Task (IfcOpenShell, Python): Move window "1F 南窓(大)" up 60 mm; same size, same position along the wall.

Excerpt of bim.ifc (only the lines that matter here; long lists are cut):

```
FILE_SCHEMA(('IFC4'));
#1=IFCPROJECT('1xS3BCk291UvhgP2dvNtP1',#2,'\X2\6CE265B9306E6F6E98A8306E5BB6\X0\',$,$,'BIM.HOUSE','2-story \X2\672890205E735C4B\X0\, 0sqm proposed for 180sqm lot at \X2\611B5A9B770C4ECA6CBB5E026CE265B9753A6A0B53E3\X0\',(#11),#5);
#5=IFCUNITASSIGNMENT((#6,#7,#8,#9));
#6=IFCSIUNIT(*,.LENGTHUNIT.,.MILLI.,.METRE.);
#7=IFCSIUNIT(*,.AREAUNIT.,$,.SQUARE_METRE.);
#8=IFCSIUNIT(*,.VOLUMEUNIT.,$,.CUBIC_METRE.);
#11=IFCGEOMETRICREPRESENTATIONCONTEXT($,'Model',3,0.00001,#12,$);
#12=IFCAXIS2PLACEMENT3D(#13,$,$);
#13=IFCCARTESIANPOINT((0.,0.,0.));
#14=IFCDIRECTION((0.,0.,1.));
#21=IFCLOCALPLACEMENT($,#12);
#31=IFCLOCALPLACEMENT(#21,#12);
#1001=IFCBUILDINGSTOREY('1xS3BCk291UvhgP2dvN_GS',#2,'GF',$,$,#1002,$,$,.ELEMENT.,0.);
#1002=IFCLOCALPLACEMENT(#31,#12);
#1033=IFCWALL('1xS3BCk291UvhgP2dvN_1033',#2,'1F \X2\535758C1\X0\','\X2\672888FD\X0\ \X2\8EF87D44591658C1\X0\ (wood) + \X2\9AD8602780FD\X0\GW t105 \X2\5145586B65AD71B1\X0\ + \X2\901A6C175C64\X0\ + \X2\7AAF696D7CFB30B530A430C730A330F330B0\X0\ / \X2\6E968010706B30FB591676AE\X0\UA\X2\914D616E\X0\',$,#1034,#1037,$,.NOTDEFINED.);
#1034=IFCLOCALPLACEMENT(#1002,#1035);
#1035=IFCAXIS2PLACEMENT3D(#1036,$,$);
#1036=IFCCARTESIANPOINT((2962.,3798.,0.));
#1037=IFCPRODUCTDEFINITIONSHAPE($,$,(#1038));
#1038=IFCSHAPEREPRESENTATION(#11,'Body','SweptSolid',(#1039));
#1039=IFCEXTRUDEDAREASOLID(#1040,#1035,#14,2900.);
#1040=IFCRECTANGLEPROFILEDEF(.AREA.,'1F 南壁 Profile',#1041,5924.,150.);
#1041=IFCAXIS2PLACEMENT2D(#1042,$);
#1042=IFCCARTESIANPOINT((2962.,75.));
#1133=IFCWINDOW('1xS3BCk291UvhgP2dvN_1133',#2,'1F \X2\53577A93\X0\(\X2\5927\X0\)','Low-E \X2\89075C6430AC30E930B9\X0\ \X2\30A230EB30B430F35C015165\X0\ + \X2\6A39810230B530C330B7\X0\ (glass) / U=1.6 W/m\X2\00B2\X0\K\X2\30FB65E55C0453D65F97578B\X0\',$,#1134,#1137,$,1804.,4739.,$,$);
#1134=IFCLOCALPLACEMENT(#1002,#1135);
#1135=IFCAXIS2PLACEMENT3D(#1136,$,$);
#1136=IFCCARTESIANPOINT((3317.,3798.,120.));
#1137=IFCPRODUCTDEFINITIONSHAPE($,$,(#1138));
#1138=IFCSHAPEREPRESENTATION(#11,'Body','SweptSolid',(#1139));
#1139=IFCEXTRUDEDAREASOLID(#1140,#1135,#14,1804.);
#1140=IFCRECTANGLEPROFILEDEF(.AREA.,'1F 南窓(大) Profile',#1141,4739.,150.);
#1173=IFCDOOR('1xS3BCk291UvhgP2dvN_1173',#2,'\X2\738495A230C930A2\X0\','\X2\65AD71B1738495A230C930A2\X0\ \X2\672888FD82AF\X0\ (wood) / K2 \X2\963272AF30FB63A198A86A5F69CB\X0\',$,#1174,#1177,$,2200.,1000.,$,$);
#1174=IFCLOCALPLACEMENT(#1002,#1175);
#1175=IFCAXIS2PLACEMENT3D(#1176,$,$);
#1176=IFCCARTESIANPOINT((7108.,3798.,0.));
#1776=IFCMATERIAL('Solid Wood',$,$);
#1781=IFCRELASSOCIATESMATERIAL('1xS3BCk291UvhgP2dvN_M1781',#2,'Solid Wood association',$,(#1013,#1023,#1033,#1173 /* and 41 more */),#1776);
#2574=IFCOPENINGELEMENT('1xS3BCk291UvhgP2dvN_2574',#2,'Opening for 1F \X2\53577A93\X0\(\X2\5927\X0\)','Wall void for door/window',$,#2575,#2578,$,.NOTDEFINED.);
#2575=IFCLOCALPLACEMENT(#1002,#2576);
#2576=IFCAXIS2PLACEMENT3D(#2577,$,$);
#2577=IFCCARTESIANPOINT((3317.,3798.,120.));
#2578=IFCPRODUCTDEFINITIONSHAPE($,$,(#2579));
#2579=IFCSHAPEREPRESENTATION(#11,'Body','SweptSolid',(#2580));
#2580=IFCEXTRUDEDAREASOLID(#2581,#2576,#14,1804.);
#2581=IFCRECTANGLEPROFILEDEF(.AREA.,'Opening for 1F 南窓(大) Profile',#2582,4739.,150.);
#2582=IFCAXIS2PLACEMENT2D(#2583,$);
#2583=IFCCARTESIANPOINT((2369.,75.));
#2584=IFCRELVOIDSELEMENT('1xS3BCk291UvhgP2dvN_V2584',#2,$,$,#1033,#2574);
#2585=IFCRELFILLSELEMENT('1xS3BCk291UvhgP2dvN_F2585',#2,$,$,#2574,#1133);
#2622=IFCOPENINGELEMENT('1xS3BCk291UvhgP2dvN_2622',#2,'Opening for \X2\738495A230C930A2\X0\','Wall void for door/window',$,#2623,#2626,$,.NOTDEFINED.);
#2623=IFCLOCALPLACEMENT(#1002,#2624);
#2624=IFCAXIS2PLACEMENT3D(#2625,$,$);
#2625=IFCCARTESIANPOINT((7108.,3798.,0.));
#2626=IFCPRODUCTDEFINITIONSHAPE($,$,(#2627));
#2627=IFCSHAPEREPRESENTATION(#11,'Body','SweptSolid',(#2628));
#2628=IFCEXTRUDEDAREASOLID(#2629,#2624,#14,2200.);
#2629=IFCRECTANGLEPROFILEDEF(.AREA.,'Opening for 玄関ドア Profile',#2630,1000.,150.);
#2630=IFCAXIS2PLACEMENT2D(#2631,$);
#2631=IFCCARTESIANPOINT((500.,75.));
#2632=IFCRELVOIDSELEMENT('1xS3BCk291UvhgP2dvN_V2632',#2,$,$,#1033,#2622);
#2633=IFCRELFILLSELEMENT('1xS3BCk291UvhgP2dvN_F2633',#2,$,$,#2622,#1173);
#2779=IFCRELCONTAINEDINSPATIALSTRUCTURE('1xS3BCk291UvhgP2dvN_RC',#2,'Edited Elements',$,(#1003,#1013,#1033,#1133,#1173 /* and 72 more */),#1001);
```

```python
import numpy as np
import ifcopenshell
import ifcopenshell.api.geometry
import ifcopenshell.util.placement
import ifcopenshell.util.unit

model = ifcopenshell.open("bim.ifc")
unit_scale = ifcopenshell.util.unit.calculate_unit_scale(model)

window = model.by_guid("1xS3BCk291UvhgP2dvN_1133")
opening = window.FillsVoids[0].RelatingOpeningElement
dz = 0.06 / unit_scale

shift = np.array([0.0, 0.0, dz])
# The window is not placed relative to its opening, so move both.
for product in (opening, window):
    matrix = ifcopenshell.util.placement.get_local_placement(product.ObjectPlacement)
    matrix[:3, 3] += shift
    ifcopenshell.api.geometry.edit_object_placement(model, product=product, matrix=matrix, is_si=False)

print(f"moved by {dz * unit_scale:+.3f} m")

model.write("bim_rev.ifc")
```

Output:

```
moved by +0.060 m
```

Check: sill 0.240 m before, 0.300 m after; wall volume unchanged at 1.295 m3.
